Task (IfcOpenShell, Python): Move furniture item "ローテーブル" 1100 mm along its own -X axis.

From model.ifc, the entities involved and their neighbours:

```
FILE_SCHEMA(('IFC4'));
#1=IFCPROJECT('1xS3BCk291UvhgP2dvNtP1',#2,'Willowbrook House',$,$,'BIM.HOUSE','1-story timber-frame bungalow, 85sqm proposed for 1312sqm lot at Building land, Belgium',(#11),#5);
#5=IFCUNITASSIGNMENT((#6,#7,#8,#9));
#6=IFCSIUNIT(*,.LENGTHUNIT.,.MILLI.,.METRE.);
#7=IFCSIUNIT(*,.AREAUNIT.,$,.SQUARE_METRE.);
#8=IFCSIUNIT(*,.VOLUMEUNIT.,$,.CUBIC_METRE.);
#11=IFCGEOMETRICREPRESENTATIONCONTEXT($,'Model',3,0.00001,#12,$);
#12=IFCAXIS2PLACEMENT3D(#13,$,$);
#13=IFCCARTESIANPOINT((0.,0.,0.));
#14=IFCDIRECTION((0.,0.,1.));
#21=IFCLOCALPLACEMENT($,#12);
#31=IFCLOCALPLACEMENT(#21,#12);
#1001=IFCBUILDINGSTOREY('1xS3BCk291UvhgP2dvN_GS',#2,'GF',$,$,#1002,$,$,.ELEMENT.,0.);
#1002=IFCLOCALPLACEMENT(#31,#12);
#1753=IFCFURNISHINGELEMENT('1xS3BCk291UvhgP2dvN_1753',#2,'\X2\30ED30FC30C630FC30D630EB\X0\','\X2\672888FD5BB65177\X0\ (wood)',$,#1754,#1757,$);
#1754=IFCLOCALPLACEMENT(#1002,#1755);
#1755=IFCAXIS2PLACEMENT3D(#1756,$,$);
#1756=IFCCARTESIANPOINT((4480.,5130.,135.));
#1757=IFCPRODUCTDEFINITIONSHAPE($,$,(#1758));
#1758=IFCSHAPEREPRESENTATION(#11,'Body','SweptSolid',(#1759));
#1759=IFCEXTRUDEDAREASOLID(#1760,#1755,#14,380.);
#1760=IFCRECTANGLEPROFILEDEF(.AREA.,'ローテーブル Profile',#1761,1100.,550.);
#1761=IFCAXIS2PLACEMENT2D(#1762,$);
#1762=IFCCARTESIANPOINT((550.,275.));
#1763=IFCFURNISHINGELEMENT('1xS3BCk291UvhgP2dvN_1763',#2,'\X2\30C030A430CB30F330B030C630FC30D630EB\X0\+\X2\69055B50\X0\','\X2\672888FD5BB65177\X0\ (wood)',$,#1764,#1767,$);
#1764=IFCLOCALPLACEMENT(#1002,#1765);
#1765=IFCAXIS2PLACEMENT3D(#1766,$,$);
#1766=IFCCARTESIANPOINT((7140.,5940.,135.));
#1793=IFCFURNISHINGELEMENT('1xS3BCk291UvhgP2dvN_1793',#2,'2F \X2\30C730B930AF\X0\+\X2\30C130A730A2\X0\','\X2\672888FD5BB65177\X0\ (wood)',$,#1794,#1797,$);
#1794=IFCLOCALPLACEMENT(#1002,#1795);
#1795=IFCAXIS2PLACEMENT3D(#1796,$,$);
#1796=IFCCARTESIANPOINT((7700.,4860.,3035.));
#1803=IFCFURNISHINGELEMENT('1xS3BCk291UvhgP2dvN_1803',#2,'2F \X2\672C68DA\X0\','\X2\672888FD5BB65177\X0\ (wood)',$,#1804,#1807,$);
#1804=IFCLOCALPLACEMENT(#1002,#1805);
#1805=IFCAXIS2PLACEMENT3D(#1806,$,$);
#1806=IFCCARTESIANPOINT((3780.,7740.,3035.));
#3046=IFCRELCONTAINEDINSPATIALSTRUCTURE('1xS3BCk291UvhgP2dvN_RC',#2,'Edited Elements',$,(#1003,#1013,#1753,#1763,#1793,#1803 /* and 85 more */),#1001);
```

```python
import ifcopenshell
import ifcopenshell.api.geometry
import ifcopenshell.util.placement
import ifcopenshell.util.unit

model = ifcopenshell.open("model.ifc")
unit_scale = ifcopenshell.util.unit.calculate_unit_scale(model)

item = model.by_guid("1xS3BCk291UvhgP2dvN_1753")
matrix = ifcopenshell.util.placement.get_local_placement(item.ObjectPlacement)
matrix[:3, 3] -= matrix[:3, 0] * 1.1 / unit_scale
ifcopenshell.api.geometry.edit_object_placement(model, product=item, matrix=matrix, is_si=False)

print(ifcopenshell.util.placement.get_local_placement(item.ObjectPlacement).round(3) + 0.0)

model.write("model_edited.ifc")
```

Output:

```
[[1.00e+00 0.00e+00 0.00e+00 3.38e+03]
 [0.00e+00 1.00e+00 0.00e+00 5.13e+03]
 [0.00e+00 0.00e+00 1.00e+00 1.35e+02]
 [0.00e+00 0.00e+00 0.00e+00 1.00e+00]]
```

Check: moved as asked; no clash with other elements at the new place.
